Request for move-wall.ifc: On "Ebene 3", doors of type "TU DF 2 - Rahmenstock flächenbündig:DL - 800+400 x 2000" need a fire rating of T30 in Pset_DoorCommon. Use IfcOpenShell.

First a look at what the model holds.

```python
import ifcopenshell
import ifcopenshell.util.element

model = ifcopenshell.open("move-wall.ifc")
print(model.schema)
storey = next(s for s in model.by_type("IfcBuildingStorey") if s.Name == "Ebene 3")
doors = [e for e in ifcopenshell.util.element.get_decomposition(storey) if e.is_a("IfcDoor")]
seen = {}
for e in doors:
    element_type = ifcopenshell.util.element.get_type(e)
    key = (element_type.Name if element_type != e and element_type else None, ifcopenshell.util.element.get_pset(e, "Pset_DoorCommon", "FireRating"))
    seen[key] = seen.get(key, 0) + 1
for (name, value), count in sorted(seen.items(), key=str):
    print(count, "x", name, "|", value)
```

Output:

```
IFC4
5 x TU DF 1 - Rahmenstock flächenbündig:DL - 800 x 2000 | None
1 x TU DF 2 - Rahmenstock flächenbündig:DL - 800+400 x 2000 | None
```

```python
import ifcopenshell
import ifcopenshell.api.pset
import ifcopenshell.util.element

model = ifcopenshell.open("move-wall.ifc")

storey = next(s for s in model.by_type("IfcBuildingStorey") if s.Name == "Ebene 3")
doors = [e for e in ifcopenshell.util.element.get_decomposition(storey) if e.is_a("IfcDoor")]

count = 0
for e in doors:
    element_type = ifcopenshell.util.element.get_type(e)
    if element_type in (None, e) or element_type.Name != "TU DF 2 - Rahmenstock flächenbündig:DL - 800+400 x 2000":
        continue
    # add_pset returns the element's existing set when there is one.
    pset = ifcopenshell.api.pset.add_pset(model, product=e, name="Pset_DoorCommon")
    ifcopenshell.api.pset.edit_pset(model, pset=pset, properties={"FireRating": "T30"})
    count += 1

print(count, "doors updated")

model.write("move-wall_v2.ifc")
```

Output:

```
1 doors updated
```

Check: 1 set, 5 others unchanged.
